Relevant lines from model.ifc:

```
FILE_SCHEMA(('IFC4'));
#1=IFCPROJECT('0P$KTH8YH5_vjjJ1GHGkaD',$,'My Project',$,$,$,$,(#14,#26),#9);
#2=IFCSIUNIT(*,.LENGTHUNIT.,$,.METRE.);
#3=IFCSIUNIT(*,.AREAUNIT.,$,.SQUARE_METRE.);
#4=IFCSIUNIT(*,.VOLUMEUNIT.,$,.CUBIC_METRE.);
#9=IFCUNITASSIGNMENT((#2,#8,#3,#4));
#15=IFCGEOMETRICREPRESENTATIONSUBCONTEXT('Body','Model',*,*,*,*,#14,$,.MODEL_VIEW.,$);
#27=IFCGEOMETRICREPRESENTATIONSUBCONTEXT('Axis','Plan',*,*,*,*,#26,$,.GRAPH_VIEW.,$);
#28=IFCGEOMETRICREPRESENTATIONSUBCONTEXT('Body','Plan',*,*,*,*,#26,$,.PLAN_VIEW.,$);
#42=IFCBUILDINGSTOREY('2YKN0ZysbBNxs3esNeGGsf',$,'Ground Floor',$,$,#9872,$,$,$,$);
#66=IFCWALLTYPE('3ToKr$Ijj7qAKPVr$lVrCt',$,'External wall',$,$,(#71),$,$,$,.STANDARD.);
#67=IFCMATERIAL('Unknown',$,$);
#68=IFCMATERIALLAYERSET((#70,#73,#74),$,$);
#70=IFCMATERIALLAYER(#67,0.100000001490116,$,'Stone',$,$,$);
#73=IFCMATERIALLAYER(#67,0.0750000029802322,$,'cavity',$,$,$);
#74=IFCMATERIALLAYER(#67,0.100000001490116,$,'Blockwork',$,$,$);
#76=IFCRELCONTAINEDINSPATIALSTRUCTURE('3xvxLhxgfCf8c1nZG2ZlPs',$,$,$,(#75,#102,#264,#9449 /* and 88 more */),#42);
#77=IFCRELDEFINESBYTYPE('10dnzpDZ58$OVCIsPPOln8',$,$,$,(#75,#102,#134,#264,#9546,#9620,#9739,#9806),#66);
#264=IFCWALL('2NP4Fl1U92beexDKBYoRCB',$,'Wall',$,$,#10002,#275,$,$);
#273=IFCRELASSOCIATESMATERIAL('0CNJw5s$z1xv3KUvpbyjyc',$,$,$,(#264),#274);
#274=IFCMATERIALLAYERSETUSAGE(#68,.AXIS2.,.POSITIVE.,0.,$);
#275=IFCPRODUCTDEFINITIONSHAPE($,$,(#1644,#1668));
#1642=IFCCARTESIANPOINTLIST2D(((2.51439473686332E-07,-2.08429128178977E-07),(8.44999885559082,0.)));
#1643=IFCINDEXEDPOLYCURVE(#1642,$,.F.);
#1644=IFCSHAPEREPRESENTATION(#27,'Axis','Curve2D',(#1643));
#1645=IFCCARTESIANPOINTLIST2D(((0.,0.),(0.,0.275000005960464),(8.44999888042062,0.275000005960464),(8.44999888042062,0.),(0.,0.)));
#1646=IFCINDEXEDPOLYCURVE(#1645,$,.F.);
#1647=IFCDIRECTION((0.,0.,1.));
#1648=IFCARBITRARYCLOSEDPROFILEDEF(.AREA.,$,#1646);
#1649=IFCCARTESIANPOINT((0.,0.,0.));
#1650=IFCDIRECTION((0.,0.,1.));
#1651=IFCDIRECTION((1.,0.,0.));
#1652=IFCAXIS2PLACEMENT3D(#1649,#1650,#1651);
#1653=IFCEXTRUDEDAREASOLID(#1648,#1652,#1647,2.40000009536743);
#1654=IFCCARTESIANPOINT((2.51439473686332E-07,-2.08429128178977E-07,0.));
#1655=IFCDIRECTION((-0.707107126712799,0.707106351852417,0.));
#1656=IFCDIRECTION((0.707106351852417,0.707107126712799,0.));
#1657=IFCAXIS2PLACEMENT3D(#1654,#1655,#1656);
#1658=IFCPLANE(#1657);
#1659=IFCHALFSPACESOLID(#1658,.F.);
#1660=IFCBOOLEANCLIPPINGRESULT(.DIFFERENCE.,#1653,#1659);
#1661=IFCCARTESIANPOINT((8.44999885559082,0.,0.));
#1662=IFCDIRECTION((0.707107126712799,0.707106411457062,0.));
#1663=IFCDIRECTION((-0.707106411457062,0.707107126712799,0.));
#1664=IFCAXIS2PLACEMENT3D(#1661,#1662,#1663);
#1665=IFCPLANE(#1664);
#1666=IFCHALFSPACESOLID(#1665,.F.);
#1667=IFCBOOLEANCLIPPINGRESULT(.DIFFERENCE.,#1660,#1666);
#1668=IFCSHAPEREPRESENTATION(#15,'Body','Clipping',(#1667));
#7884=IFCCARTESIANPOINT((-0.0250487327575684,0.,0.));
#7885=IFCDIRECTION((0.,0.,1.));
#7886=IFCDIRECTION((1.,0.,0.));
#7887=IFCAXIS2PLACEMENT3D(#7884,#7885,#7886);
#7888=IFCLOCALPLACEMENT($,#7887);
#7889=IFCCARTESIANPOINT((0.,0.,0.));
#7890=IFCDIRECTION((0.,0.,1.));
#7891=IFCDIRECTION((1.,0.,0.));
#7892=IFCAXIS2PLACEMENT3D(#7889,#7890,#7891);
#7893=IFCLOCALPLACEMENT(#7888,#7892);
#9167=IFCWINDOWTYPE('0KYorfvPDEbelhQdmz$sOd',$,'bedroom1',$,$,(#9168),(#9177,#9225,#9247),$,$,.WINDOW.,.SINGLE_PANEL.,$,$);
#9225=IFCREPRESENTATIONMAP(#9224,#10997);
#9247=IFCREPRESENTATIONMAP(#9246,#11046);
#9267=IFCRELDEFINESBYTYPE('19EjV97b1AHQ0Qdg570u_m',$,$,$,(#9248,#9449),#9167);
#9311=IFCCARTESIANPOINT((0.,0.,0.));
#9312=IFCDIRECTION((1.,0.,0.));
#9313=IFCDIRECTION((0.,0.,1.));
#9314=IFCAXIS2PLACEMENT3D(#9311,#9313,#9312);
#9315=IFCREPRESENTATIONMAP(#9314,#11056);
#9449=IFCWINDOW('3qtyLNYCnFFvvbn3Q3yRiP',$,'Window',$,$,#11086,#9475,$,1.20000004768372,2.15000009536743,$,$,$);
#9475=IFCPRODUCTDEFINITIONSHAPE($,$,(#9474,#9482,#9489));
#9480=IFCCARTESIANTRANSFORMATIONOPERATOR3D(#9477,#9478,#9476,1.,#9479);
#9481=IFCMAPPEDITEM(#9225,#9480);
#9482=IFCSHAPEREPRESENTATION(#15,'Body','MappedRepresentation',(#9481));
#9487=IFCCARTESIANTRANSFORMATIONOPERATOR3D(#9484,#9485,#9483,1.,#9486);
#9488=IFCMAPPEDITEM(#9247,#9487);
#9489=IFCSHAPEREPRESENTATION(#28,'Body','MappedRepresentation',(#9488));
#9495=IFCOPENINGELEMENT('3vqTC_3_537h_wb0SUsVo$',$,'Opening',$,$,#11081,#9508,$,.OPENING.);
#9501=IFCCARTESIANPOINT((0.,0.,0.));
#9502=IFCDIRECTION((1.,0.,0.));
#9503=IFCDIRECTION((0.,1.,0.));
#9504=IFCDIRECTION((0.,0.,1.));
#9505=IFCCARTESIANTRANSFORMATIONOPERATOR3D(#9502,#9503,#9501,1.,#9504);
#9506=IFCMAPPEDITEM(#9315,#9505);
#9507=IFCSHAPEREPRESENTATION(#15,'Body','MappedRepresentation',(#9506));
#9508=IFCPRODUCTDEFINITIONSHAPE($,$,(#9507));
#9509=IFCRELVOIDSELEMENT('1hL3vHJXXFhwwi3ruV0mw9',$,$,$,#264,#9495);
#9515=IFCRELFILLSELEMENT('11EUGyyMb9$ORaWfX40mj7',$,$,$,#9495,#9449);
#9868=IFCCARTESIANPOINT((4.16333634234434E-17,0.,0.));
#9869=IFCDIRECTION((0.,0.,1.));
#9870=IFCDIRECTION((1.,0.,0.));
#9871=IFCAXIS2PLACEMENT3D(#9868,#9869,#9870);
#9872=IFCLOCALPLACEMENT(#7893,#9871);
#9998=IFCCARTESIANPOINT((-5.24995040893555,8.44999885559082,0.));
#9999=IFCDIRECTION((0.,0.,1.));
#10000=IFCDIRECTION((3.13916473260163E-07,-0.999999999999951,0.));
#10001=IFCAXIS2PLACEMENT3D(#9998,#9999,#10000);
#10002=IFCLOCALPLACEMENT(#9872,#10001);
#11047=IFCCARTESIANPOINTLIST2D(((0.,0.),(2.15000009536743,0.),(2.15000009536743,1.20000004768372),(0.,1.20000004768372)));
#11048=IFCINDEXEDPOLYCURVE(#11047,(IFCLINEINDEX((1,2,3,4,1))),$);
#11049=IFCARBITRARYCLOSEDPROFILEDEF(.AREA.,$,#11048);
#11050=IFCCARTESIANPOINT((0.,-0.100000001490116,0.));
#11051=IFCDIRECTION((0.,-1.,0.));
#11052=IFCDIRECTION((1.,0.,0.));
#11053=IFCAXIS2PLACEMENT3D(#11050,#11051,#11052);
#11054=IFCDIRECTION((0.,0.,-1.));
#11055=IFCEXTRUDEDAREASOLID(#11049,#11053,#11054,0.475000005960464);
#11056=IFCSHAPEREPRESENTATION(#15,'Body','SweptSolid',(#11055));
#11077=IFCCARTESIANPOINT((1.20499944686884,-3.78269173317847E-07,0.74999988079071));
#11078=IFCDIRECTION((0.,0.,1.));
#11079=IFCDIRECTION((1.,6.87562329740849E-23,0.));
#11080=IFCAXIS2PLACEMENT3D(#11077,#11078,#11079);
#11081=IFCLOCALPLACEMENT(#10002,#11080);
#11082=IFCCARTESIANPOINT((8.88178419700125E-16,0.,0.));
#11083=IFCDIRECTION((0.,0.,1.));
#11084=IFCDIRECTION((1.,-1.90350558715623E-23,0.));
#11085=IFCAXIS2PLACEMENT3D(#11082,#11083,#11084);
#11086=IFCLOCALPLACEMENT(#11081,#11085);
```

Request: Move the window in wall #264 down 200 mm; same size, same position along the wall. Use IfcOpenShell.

```python
import numpy as np
import ifcopenshell
import ifcopenshell.api.geometry
import ifcopenshell.util.placement
import ifcopenshell.util.unit

model = ifcopenshell.open("model.ifc")
unit_scale = ifcopenshell.util.unit.calculate_unit_scale(model)

window = model.by_id(9449)
opening = window.FillsVoids[0].RelatingOpeningElement
dz = -0.2 / unit_scale

shift = np.array([0.0, 0.0, dz])
# The window is placed relative to its opening, so it follows when the opening moves.
matrix = ifcopenshell.util.placement.get_local_placement(opening.ObjectPlacement)
matrix[:3, 3] += shift
ifcopenshell.api.geometry.edit_object_placement(
    model, product=opening, matrix=matrix, is_si=False, should_transform_children=True
)

print(f"moved by {dz * unit_scale:+.3f} m")

model.write("model_v2.ifc")
```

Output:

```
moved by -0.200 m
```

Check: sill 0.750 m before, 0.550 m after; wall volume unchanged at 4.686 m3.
